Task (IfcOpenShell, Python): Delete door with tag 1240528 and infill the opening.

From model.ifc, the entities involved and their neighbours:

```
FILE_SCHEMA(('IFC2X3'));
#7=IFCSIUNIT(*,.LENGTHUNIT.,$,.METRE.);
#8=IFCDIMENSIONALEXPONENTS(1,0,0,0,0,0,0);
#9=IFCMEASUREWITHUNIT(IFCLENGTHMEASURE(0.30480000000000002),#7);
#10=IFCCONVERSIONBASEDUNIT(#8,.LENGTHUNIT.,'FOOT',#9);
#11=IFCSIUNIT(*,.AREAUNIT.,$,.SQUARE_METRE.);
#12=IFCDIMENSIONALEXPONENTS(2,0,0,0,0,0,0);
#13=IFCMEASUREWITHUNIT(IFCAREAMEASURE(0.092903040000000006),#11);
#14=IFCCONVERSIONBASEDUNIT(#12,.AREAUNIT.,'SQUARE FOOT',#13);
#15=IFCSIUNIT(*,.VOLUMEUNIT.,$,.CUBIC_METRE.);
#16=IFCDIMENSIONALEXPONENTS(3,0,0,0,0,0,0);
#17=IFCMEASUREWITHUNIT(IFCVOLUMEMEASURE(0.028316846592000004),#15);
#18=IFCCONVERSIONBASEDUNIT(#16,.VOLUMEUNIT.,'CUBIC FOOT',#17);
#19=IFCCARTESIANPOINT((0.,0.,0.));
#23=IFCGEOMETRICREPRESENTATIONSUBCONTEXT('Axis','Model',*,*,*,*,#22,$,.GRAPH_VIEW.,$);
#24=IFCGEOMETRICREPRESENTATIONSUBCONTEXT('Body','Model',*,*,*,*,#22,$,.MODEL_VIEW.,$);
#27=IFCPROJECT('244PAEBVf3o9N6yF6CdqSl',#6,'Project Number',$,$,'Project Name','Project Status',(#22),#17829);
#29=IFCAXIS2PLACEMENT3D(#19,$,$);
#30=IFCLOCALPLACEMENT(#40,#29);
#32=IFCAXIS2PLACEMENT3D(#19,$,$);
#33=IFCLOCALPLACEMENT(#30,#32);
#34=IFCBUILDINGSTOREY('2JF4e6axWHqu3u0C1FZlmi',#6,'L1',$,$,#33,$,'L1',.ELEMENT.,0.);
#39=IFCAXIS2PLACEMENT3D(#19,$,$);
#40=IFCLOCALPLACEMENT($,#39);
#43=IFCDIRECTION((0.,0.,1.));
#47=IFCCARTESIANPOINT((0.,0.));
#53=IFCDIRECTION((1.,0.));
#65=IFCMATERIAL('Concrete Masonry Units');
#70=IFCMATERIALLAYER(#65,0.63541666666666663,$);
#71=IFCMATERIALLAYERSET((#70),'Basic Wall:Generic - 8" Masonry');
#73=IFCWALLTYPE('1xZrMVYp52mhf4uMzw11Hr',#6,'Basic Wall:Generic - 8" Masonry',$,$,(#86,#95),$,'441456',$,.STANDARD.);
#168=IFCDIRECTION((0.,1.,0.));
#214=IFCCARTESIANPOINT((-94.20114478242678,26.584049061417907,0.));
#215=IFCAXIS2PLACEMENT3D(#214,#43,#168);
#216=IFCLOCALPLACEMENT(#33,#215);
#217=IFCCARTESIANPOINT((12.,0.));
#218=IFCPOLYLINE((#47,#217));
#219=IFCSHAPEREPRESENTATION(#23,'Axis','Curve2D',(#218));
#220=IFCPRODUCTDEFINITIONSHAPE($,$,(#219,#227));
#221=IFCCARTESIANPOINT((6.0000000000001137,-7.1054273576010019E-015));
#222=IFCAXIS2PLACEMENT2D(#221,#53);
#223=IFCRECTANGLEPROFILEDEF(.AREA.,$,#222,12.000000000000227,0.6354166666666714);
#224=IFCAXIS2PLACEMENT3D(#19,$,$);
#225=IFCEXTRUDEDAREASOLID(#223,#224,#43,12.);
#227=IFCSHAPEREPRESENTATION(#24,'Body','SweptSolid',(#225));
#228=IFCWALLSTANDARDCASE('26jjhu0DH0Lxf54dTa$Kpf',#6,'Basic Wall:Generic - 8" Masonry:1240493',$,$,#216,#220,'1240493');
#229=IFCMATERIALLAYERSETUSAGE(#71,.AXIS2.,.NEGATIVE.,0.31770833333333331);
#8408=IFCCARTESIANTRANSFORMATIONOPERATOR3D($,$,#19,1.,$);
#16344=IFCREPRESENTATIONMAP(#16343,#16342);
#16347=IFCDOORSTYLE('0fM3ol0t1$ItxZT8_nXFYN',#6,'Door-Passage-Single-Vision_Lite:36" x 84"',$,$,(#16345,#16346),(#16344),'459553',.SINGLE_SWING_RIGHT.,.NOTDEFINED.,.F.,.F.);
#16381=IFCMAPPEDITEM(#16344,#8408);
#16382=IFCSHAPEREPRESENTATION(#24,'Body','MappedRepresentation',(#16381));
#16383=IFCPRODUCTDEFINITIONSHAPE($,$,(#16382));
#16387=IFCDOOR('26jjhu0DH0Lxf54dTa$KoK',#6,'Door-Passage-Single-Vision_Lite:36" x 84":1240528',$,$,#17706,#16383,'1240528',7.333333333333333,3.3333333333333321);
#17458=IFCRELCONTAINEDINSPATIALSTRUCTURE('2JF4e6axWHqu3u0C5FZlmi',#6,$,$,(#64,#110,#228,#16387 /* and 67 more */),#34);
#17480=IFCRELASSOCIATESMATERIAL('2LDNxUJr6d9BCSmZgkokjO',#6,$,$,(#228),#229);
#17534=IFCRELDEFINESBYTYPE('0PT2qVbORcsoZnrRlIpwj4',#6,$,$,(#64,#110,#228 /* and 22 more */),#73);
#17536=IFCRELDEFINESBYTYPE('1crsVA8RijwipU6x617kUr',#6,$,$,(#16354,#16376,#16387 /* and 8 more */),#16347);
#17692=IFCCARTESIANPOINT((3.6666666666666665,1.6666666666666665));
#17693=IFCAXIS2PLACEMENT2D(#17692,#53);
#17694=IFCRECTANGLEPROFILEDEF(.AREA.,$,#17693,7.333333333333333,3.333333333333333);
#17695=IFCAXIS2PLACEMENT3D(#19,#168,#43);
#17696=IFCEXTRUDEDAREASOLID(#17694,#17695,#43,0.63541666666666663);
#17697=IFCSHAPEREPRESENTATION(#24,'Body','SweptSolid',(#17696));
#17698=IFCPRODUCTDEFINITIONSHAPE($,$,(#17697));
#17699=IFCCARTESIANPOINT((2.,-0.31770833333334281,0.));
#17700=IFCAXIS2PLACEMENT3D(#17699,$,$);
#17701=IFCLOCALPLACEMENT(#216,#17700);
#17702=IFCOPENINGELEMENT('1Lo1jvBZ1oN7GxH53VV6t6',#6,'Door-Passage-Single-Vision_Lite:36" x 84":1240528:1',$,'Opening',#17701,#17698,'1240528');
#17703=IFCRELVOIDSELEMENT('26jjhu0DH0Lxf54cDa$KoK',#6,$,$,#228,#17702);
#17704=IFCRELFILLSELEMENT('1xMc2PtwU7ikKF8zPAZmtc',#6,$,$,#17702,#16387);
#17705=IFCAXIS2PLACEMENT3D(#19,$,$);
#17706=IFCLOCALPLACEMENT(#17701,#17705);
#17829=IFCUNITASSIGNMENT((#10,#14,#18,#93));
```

```python
import ifcopenshell
import ifcopenshell.api.feature
import ifcopenshell.api.root
import ifcopenshell.geom
import ifcopenshell.util.shape

model = ifcopenshell.open("model.ifc")
settings = ifcopenshell.geom.settings()


def volume(element):
    """Net volume in cubic metres, openings subtracted."""
    shape = ifcopenshell.geom.create_shape(settings, element)
    return ifcopenshell.util.shape.get_volume(shape.geometry)


door = model.by_id(16387)
opening = door.FillsVoids[0].RelatingOpeningElement
wall = opening.VoidsElements[0].RelatingBuildingElement
before = volume(wall)

ifcopenshell.api.root.remove_product(model, product=door)
ifcopenshell.api.feature.remove_feature(model, feature=opening)

after = volume(wall)

print(f"wall volume {before:.3f} -> {after:.3f} m3")

model.write("model_rev.ifc")
```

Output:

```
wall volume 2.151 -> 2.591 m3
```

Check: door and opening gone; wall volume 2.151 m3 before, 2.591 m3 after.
